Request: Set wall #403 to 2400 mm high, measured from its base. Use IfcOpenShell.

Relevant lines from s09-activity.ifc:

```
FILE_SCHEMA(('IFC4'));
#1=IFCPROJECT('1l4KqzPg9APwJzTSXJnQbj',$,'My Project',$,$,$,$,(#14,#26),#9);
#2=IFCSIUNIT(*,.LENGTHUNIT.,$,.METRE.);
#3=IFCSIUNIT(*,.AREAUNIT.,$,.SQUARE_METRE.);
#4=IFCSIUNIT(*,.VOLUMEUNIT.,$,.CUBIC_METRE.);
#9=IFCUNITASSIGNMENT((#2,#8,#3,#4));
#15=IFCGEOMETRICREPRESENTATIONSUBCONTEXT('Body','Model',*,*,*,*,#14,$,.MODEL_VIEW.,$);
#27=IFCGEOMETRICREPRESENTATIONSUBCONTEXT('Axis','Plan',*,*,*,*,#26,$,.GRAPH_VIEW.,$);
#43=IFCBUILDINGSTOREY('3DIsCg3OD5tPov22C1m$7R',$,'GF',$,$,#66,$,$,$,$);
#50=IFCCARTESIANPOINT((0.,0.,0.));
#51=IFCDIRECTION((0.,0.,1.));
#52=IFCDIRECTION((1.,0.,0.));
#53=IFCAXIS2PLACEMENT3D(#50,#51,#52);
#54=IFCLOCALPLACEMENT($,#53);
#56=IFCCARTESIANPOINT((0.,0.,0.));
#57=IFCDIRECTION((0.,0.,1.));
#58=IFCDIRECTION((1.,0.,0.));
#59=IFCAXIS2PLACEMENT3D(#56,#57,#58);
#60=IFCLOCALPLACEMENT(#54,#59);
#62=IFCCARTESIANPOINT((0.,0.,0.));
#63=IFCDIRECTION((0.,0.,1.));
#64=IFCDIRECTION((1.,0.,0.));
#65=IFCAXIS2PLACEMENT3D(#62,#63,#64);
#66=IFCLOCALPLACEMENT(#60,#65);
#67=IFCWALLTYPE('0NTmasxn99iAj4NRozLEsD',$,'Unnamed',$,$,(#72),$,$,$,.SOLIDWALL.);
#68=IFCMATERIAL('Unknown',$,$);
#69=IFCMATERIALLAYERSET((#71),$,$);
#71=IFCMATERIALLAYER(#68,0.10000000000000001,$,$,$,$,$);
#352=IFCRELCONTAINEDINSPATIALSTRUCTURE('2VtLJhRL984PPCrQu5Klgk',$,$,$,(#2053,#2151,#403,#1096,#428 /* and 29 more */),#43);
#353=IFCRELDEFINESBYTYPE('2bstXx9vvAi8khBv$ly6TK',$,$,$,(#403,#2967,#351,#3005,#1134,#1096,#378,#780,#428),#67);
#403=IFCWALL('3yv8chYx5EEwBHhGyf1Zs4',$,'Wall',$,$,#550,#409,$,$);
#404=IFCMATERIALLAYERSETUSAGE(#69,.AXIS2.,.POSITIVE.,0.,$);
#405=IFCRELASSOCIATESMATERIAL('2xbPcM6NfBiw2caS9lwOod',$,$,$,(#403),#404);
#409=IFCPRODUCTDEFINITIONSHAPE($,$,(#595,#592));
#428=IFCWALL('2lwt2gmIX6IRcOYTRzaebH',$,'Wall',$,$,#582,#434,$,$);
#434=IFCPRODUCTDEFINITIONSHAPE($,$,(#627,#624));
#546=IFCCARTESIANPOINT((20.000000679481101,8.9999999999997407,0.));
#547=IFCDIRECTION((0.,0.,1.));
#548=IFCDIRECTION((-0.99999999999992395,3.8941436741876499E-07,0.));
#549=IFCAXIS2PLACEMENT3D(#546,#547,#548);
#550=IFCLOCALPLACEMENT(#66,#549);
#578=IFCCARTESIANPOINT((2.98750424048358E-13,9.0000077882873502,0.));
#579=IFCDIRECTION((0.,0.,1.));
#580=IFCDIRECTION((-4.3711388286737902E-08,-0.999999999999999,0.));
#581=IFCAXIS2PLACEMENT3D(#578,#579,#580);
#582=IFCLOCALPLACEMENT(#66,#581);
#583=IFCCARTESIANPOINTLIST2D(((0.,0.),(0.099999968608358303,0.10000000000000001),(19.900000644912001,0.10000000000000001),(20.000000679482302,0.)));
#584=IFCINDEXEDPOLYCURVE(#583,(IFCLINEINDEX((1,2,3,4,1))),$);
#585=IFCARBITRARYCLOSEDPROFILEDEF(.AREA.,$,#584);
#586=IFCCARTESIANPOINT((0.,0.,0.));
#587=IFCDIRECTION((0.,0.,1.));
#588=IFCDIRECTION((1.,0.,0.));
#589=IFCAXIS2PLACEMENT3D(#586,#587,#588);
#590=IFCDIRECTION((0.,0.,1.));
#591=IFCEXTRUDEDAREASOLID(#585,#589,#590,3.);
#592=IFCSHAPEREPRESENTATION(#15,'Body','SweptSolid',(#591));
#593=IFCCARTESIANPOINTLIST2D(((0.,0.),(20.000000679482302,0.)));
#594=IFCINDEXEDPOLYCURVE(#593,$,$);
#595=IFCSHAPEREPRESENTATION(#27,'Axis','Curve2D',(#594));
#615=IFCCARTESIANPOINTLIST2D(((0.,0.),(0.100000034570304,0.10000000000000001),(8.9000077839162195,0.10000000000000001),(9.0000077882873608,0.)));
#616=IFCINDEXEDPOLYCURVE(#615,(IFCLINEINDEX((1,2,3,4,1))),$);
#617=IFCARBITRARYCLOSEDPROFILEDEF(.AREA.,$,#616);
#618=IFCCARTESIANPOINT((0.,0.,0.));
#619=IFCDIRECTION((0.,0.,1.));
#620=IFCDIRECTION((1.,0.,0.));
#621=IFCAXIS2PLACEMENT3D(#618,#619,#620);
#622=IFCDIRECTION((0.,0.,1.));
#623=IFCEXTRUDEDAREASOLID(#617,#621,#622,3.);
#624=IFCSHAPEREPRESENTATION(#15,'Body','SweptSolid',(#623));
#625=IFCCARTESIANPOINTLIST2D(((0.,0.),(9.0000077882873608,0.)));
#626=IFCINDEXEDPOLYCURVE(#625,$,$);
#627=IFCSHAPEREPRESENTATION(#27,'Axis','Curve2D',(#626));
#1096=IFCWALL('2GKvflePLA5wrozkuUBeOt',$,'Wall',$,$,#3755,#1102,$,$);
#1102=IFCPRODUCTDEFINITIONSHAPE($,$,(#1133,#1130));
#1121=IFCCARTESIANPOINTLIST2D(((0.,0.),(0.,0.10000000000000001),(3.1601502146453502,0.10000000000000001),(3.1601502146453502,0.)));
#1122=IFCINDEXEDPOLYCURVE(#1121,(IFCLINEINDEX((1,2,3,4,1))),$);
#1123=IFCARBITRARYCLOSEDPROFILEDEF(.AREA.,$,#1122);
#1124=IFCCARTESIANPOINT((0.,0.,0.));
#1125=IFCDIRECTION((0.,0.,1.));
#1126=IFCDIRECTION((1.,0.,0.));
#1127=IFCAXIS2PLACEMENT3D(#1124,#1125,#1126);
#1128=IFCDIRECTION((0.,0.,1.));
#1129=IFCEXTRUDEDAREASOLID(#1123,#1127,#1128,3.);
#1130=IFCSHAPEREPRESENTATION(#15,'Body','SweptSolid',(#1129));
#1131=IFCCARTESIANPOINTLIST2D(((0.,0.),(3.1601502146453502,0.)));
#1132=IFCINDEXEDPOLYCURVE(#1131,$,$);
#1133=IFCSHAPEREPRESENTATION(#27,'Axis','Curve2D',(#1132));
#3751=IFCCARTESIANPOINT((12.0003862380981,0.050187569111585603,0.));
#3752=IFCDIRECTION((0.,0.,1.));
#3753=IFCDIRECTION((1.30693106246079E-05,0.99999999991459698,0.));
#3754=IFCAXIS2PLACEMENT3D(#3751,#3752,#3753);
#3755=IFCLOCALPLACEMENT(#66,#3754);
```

```python
import ifcopenshell
import ifcopenshell.geom
import ifcopenshell.util.representation
import ifcopenshell.util.shape
import ifcopenshell.util.unit

model = ifcopenshell.open("s09-activity.ifc")
unit_scale = ifcopenshell.util.unit.calculate_unit_scale(model)
settings = ifcopenshell.geom.settings()


def volume(element):
    """Net volume in cubic metres, openings subtracted."""
    shape = ifcopenshell.geom.create_shape(settings, element)
    return ifcopenshell.util.shape.get_volume(shape.geometry)


wall = model.by_id(403)
before = volume(wall)

body = ifcopenshell.util.representation.get_representation(wall, "Model", "Body")
solid = body.Items[0]
old_height = solid.Depth
solid.Depth = 2.4 / unit_scale
after = volume(wall)

print(f"height {old_height:g} -> {solid.Depth:g}, volume {before:.3f} -> {after:.3f} m3")

model.write("s09-activity_updated.ifc")
```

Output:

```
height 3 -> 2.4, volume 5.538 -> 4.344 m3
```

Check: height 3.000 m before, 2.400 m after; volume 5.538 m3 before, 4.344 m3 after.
